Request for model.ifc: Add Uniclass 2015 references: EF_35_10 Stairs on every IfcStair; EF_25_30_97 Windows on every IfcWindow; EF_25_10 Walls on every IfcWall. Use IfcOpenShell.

First a look at what the model holds.

```python
import ifcopenshell

model = ifcopenshell.open("model.ifc")
print(model.schema)
print("classifications:", [c.Name for c in model.by_type("IfcClassification")])
for ifc_class in ("IfcDoor", "IfcRoof", "IfcStair", "IfcWall", "IfcWindow"):
    print(ifc_class, len(model.by_type(ifc_class)))
```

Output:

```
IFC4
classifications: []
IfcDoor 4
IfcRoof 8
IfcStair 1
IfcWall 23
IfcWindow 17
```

```python
import ifcopenshell
import ifcopenshell.api.classification

model = ifcopenshell.open("model.ifc")

system = ifcopenshell.api.classification.add_classification(model, classification="Uniclass 2015")

codes = {
    "IfcStair": ("EF_35_10", "Stairs"),
    "IfcWindow": ("EF_25_30_97", "Windows"),
    "IfcWall": ("EF_25_10", "Walls"),
}
for ifc_class, (code, name) in codes.items():
    products = model.by_type(ifc_class)
    ifcopenshell.api.classification.add_reference(
        model, products=products, classification=system, identification=code, name=name
    )
    print(code, len(products))

model.write("model-out.ifc")
```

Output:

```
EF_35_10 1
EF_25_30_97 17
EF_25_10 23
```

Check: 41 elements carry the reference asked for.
